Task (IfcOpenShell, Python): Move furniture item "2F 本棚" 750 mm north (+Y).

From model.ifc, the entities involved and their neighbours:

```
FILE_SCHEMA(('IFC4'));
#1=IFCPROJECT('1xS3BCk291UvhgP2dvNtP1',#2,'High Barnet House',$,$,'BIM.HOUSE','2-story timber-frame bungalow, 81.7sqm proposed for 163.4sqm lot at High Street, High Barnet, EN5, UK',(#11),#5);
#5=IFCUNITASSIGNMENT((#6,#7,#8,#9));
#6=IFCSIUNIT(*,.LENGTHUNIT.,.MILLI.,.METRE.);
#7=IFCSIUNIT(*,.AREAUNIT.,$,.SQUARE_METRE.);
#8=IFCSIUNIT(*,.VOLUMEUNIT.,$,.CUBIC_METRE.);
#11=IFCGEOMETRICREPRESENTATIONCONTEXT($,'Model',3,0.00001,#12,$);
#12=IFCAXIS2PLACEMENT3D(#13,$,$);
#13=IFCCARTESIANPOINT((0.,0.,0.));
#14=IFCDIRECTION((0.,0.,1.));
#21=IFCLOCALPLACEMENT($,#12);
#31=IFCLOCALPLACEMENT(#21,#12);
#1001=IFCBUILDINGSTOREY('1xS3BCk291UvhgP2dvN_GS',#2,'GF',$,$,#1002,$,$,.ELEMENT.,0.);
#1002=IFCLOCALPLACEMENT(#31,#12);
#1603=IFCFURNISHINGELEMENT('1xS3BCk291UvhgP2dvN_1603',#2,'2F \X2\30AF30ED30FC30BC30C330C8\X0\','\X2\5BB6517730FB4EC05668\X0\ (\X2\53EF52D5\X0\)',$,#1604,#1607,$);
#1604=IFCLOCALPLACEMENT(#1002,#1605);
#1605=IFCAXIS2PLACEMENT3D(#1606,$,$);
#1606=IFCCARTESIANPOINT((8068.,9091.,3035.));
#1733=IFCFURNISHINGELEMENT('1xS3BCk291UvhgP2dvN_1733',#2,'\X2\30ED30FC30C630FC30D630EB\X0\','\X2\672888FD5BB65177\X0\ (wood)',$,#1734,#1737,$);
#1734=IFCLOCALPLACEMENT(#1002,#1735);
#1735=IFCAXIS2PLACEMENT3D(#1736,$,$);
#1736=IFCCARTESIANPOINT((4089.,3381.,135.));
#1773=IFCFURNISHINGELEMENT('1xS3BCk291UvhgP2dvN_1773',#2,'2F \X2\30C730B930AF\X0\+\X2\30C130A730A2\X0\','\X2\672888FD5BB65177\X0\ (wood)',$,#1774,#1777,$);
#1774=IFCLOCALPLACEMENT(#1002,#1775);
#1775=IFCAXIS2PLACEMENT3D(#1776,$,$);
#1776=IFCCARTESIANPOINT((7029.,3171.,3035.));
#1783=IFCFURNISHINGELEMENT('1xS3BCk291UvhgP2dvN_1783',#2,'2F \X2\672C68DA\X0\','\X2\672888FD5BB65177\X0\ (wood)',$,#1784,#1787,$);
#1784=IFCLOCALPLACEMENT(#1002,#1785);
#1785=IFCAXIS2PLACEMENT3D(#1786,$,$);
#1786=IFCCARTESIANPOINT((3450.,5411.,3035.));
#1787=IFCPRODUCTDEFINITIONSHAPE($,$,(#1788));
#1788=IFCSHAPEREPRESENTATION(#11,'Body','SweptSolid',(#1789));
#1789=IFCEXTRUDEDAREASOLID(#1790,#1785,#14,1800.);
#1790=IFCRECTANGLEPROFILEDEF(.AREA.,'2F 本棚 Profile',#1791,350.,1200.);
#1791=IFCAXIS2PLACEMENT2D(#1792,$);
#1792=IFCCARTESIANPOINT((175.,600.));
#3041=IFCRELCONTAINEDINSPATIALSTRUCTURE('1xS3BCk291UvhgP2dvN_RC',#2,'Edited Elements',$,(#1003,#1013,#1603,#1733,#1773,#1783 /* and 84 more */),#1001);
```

```python
import ifcopenshell
import ifcopenshell.api.geometry
import ifcopenshell.util.placement
import ifcopenshell.util.unit

model = ifcopenshell.open("model.ifc")
unit_scale = ifcopenshell.util.unit.calculate_unit_scale(model)

item = model.by_guid("1xS3BCk291UvhgP2dvN_1783")
matrix = ifcopenshell.util.placement.get_local_placement(item.ObjectPlacement)
matrix[1, 3] += 0.75 / unit_scale
ifcopenshell.api.geometry.edit_object_placement(model, product=item, matrix=matrix, is_si=False)

print(ifcopenshell.util.placement.get_local_placement(item.ObjectPlacement).round(3) + 0.0)

model.write("model_v2.ifc")
```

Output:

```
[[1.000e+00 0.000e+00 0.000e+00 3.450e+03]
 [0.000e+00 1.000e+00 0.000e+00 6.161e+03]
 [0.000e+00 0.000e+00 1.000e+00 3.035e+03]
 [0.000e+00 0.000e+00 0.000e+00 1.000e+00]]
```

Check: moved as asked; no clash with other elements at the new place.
